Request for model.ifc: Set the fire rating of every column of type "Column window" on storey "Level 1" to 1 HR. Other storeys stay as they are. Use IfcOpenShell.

First a look at what the model holds.

```python
import ifcopenshell
import ifcopenshell.util.element

model = ifcopenshell.open("model.ifc")
print(model.schema)
storey = next(s for s in model.by_type("IfcBuildingStorey") if s.Name == "Level 1")
columns = [e for e in ifcopenshell.util.element.get_decomposition(storey) if e.is_a("IfcColumn")]
seen = {}
for e in columns:
    element_type = ifcopenshell.util.element.get_type(e)
    key = (element_type.Name if element_type != e and element_type else None, ifcopenshell.util.element.get_pset(e, "Pset_ColumnCommon", "FireRating"))
    seen[key] = seen.get(key, 0) + 1
for (name, value), count in sorted(seen.items(), key=str):
    print(count, "x", name, "|", value)
```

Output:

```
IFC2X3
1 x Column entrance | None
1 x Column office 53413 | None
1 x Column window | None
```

```python
import ifcopenshell
import ifcopenshell.api.pset
import ifcopenshell.util.element

model = ifcopenshell.open("model.ifc")

storey = next(s for s in model.by_type("IfcBuildingStorey") if s.Name == "Level 1")
columns = [e for e in ifcopenshell.util.element.get_decomposition(storey) if e.is_a("IfcColumn")]

count = 0
for e in columns:
    element_type = ifcopenshell.util.element.get_type(e)
    if element_type in (None, e) or element_type.Name != "Column window":
        continue
    # add_pset returns the element's existing set when there is one.
    pset = ifcopenshell.api.pset.add_pset(model, product=e, name="Pset_ColumnCommon")
    ifcopenshell.api.pset.edit_pset(model, pset=pset, properties={"FireRating": "1 HR"})
    count += 1

print(count, "columns updated")

model.write("model_v2.ifc")
```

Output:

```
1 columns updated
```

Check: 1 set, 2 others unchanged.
